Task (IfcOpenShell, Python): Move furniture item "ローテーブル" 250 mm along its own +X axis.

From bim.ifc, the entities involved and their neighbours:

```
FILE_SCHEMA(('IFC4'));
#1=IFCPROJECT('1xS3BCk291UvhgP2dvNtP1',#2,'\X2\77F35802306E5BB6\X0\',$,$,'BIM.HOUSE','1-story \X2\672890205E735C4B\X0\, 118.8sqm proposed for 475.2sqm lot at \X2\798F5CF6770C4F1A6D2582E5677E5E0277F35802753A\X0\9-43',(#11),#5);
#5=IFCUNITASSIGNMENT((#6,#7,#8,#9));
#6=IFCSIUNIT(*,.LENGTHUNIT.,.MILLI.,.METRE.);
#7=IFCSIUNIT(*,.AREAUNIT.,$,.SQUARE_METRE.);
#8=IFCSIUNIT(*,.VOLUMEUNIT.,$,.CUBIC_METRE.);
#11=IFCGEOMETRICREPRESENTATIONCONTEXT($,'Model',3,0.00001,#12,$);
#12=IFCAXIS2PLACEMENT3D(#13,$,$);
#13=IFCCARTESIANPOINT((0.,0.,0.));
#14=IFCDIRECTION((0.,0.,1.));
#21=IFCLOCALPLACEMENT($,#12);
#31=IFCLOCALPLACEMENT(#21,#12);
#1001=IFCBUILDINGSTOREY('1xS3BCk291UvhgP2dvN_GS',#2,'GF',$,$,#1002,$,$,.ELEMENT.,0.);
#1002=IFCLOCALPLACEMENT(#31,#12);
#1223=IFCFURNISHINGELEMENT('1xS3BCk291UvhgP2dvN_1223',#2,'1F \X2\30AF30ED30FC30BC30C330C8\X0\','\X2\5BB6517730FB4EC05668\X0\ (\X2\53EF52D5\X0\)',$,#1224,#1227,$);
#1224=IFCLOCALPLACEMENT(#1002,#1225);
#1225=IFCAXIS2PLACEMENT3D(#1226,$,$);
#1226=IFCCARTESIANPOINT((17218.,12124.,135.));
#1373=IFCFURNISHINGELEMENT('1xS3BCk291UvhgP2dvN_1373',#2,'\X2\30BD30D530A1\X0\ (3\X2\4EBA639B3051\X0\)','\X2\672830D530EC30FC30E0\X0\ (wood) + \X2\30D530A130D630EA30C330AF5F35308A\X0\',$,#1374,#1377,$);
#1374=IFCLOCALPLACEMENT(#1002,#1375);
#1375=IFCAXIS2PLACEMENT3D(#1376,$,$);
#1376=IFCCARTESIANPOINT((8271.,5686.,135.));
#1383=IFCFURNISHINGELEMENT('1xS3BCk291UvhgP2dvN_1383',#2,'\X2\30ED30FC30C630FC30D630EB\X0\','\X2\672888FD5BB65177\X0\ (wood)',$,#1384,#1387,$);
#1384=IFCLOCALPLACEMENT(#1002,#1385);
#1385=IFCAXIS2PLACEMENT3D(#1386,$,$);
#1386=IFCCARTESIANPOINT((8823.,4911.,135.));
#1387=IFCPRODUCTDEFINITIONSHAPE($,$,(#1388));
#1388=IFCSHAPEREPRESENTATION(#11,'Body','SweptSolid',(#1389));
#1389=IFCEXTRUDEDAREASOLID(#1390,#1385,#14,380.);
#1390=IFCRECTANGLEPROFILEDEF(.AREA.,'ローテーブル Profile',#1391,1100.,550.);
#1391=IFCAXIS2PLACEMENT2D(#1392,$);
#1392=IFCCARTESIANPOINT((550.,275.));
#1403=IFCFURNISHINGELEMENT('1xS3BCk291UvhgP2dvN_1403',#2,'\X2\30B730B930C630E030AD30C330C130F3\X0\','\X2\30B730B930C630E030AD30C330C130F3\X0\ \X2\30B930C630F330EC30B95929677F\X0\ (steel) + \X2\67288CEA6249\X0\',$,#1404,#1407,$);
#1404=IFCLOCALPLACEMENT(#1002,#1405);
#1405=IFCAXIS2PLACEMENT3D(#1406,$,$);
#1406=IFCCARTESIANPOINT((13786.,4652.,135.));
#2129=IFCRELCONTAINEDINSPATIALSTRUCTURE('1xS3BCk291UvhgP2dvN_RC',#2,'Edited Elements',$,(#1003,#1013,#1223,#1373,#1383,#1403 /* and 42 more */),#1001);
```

```python
import ifcopenshell
import ifcopenshell.api.geometry
import ifcopenshell.util.placement
import ifcopenshell.util.unit

model = ifcopenshell.open("bim.ifc")
unit_scale = ifcopenshell.util.unit.calculate_unit_scale(model)

item = model.by_guid("1xS3BCk291UvhgP2dvN_1383")
matrix = ifcopenshell.util.placement.get_local_placement(item.ObjectPlacement)
matrix[:3, 3] += matrix[:3, 0] * 0.25 / unit_scale
ifcopenshell.api.geometry.edit_object_placement(model, product=item, matrix=matrix, is_si=False)

print(ifcopenshell.util.placement.get_local_placement(item.ObjectPlacement).round(3) + 0.0)

model.write("bim_updated.ifc")
```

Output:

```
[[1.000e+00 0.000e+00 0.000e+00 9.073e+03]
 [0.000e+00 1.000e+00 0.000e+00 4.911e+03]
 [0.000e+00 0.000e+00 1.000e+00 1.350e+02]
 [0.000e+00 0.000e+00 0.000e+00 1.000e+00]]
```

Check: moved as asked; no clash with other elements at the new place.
